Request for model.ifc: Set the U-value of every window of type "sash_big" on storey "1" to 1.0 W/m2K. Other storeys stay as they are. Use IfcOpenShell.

First a look at what the model holds.

```python
import ifcopenshell
import ifcopenshell.util.element

model = ifcopenshell.open("model.ifc")
print(model.schema)
storey = next(s for s in model.by_type("IfcBuildingStorey") if s.Name == "1")
windows = [e for e in ifcopenshell.util.element.get_decomposition(storey) if e.is_a("IfcWindow")]
seen = {}
for e in windows:
    element_type = ifcopenshell.util.element.get_type(e)
    key = (element_type.Name if element_type != e and element_type else None, ifcopenshell.util.element.get_pset(e, "Pset_WindowCommon", "ThermalTransmittance"))
    seen[key] = seen.get(key, 0) + 1
for (name, value), count in sorted(seen.items(), key=str):
    print(count, "x", name, "|", value)
```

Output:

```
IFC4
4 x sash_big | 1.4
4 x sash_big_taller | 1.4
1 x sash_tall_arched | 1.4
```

```python
import ifcopenshell
import ifcopenshell.api.pset
import ifcopenshell.util.element

model = ifcopenshell.open("model.ifc")

storey = next(s for s in model.by_type("IfcBuildingStorey") if s.Name == "1")
windows = [e for e in ifcopenshell.util.element.get_decomposition(storey) if e.is_a("IfcWindow")]

count = 0
for e in windows:
    element_type = ifcopenshell.util.element.get_type(e)
    if element_type in (None, e) or element_type.Name != "sash_big":
        continue
    # add_pset returns the element's existing set when there is one.
    pset = ifcopenshell.api.pset.add_pset(model, product=e, name="Pset_WindowCommon")
    ifcopenshell.api.pset.edit_pset(model, pset=pset, properties={"ThermalTransmittance": 1.0})
    count += 1

print(count, "windows updated")

model.write("model-out.ifc")
```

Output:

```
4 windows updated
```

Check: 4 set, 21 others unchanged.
